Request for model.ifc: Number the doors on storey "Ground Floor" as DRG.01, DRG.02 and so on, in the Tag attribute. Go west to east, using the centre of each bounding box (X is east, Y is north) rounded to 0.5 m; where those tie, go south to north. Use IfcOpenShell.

First a look at what the model holds.

```python
import ifcopenshell
import ifcopenshell.util.element
import ifcopenshell.util.placement

model = ifcopenshell.open("model.ifc")
print(model.schema)
storey = next(s for s in model.by_type("IfcBuildingStorey") if s.Name == "Ground Floor")
doors = [e for e in ifcopenshell.util.element.get_decomposition(storey) if e.is_a("IfcDoor")]
for e in sorted(doors, key=lambda e: e.id()):
    origin = ifcopenshell.util.placement.get_local_placement(e.ObjectPlacement)[:3, 3]
    print(e.id(), e.Tag, e.Name, origin.round(2) + 0.0, sep=" | ")
```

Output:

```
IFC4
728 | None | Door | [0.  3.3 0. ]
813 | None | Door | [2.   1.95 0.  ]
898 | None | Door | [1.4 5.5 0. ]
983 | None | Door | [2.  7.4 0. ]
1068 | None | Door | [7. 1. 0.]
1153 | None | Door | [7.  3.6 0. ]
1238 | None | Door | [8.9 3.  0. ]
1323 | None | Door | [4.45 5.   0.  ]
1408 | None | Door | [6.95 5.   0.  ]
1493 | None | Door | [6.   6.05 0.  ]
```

```python
import ifcopenshell
import ifcopenshell.geom
import ifcopenshell.util.element
import ifcopenshell.util.shape

model = ifcopenshell.open("model.ifc")
settings = ifcopenshell.geom.settings()
settings.set("use-world-coords", True)


def centre(element):
    shape = ifcopenshell.geom.create_shape(settings, element)
    return ifcopenshell.util.shape.get_bbox_centroid(shape.geometry)


storey = next(s for s in model.by_type("IfcBuildingStorey") if s.Name == "Ground Floor")
doors = [e for e in ifcopenshell.util.element.get_decomposition(storey) if e.is_a("IfcDoor")]

# Insertion points can sit at a corner or the storey origin, so sort by the geometry (in metres).
centres = {e: centre(e) for e in doors}
doors.sort(key=lambda e: (round(centres[e][0] / 0.5), centres[e][1]))

for i, e in enumerate(doors, start=1):
    number = f"DRG.{i:02d}"
    e.Tag = number
    print(e.id(), number)

model.write("model_edited.ifc")
```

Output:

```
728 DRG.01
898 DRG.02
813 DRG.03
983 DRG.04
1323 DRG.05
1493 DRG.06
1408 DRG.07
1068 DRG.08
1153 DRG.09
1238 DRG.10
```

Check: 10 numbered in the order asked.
